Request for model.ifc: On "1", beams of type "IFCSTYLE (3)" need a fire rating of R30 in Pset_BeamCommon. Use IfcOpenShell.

First a look at what the model holds.

```python
import ifcopenshell
import ifcopenshell.util.element

model = ifcopenshell.open("model.ifc")
print(model.schema)
storey = next(s for s in model.by_type("IfcBuildingStorey") if s.Name == "1")
beams = [e for e in ifcopenshell.util.element.get_decomposition(storey) if e.is_a("IfcBeam")]
seen = {}
for e in beams:
    element_type = ifcopenshell.util.element.get_type(e)
    key = (element_type.Name if element_type != e and element_type else None, ifcopenshell.util.element.get_pset(e, "Pset_BeamCommon", "FireRating"))
    seen[key] = seen.get(key, 0) + 1
for (name, value), count in sorted(seen.items(), key=str):
    print(count, "x", name, "|", value)
```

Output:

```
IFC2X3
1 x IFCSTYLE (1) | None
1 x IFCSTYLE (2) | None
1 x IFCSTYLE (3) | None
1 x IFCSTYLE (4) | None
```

```python
import ifcopenshell
import ifcopenshell.api.pset
import ifcopenshell.util.element

model = ifcopenshell.open("model.ifc")

storey = next(s for s in model.by_type("IfcBuildingStorey") if s.Name == "1")
beams = [e for e in ifcopenshell.util.element.get_decomposition(storey) if e.is_a("IfcBeam")]

count = 0
for e in beams:
    element_type = ifcopenshell.util.element.get_type(e)
    if element_type in (None, e) or element_type.Name != "IFCSTYLE (3)":
        continue
    # add_pset returns the element's existing set when there is one.
    pset = ifcopenshell.api.pset.add_pset(model, product=e, name="Pset_BeamCommon")
    ifcopenshell.api.pset.edit_pset(model, pset=pset, properties={"FireRating": "R30"})
    count += 1

print(count, "beams updated")

model.write("model_updated.ifc")
```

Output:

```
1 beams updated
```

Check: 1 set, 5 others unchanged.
